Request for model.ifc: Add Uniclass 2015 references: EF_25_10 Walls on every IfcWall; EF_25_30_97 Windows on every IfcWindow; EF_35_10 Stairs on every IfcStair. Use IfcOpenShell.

First a look at what the model holds.

```python
import ifcopenshell

model = ifcopenshell.open("model.ifc")
print(model.schema)
print("classifications:", [c.Name for c in model.by_type("IfcClassification")])
for ifc_class in ("IfcDoor", "IfcRoof", "IfcStair", "IfcWall", "IfcWindow"):
    print(ifc_class, len(model.by_type(ifc_class)))
```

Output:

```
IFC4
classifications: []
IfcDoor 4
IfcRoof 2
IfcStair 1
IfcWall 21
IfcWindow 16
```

```python
import ifcopenshell
import ifcopenshell.api.classification

model = ifcopenshell.open("model.ifc")

system = ifcopenshell.api.classification.add_classification(model, classification="Uniclass 2015")

codes = {
    "IfcWall": ("EF_25_10", "Walls"),
    "IfcWindow": ("EF_25_30_97", "Windows"),
    "IfcStair": ("EF_35_10", "Stairs"),
}
for ifc_class, (code, name) in codes.items():
    products = model.by_type(ifc_class)
    ifcopenshell.api.classification.add_reference(
        model, products=products, classification=system, identification=code, name=name
    )
    print(code, len(products))

model.write("model_updated.ifc")
```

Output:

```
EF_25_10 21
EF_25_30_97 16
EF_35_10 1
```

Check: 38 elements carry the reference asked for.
